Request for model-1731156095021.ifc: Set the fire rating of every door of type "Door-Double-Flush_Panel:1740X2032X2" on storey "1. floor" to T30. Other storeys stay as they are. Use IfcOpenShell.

First a look at what the model holds.

```python
import ifcopenshell
import ifcopenshell.util.element

model = ifcopenshell.open("model-1731156095021.ifc")
print(model.schema)
storey = next(s for s in model.by_type("IfcBuildingStorey") if s.Name == "1. floor")
doors = [e for e in ifcopenshell.util.element.get_decomposition(storey) if e.is_a("IfcDoor")]
seen = {}
for e in doors:
    element_type = ifcopenshell.util.element.get_type(e)
    key = (element_type.Name if element_type != e and element_type else None, ifcopenshell.util.element.get_pset(e, "Pset_DoorCommon", "FireRating"))
    seen[key] = seen.get(key, 0) + 1
for (name, value), count in sorted(seen.items(), key=str):
    print(count, "x", name, "|", value)
```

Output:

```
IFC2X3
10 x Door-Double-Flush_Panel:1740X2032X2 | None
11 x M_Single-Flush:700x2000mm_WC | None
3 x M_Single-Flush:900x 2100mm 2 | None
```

```python
import ifcopenshell
import ifcopenshell.api.pset
import ifcopenshell.util.element

model = ifcopenshell.open("model-1731156095021.ifc")

storey = next(s for s in model.by_type("IfcBuildingStorey") if s.Name == "1. floor")
doors = [e for e in ifcopenshell.util.element.get_decomposition(storey) if e.is_a("IfcDoor")]

count = 0
for e in doors:
    element_type = ifcopenshell.util.element.get_type(e)
    if element_type in (None, e) or element_type.Name != "Door-Double-Flush_Panel:1740X2032X2":
        continue
    # add_pset returns the element's existing set when there is one.
    pset = ifcopenshell.api.pset.add_pset(model, product=e, name="Pset_DoorCommon")
    ifcopenshell.api.pset.edit_pset(model, pset=pset, properties={"FireRating": "T30"})
    count += 1

print(count, "doors updated")

model.write("model-1731156095021_rev.ifc")
```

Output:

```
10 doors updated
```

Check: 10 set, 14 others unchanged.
